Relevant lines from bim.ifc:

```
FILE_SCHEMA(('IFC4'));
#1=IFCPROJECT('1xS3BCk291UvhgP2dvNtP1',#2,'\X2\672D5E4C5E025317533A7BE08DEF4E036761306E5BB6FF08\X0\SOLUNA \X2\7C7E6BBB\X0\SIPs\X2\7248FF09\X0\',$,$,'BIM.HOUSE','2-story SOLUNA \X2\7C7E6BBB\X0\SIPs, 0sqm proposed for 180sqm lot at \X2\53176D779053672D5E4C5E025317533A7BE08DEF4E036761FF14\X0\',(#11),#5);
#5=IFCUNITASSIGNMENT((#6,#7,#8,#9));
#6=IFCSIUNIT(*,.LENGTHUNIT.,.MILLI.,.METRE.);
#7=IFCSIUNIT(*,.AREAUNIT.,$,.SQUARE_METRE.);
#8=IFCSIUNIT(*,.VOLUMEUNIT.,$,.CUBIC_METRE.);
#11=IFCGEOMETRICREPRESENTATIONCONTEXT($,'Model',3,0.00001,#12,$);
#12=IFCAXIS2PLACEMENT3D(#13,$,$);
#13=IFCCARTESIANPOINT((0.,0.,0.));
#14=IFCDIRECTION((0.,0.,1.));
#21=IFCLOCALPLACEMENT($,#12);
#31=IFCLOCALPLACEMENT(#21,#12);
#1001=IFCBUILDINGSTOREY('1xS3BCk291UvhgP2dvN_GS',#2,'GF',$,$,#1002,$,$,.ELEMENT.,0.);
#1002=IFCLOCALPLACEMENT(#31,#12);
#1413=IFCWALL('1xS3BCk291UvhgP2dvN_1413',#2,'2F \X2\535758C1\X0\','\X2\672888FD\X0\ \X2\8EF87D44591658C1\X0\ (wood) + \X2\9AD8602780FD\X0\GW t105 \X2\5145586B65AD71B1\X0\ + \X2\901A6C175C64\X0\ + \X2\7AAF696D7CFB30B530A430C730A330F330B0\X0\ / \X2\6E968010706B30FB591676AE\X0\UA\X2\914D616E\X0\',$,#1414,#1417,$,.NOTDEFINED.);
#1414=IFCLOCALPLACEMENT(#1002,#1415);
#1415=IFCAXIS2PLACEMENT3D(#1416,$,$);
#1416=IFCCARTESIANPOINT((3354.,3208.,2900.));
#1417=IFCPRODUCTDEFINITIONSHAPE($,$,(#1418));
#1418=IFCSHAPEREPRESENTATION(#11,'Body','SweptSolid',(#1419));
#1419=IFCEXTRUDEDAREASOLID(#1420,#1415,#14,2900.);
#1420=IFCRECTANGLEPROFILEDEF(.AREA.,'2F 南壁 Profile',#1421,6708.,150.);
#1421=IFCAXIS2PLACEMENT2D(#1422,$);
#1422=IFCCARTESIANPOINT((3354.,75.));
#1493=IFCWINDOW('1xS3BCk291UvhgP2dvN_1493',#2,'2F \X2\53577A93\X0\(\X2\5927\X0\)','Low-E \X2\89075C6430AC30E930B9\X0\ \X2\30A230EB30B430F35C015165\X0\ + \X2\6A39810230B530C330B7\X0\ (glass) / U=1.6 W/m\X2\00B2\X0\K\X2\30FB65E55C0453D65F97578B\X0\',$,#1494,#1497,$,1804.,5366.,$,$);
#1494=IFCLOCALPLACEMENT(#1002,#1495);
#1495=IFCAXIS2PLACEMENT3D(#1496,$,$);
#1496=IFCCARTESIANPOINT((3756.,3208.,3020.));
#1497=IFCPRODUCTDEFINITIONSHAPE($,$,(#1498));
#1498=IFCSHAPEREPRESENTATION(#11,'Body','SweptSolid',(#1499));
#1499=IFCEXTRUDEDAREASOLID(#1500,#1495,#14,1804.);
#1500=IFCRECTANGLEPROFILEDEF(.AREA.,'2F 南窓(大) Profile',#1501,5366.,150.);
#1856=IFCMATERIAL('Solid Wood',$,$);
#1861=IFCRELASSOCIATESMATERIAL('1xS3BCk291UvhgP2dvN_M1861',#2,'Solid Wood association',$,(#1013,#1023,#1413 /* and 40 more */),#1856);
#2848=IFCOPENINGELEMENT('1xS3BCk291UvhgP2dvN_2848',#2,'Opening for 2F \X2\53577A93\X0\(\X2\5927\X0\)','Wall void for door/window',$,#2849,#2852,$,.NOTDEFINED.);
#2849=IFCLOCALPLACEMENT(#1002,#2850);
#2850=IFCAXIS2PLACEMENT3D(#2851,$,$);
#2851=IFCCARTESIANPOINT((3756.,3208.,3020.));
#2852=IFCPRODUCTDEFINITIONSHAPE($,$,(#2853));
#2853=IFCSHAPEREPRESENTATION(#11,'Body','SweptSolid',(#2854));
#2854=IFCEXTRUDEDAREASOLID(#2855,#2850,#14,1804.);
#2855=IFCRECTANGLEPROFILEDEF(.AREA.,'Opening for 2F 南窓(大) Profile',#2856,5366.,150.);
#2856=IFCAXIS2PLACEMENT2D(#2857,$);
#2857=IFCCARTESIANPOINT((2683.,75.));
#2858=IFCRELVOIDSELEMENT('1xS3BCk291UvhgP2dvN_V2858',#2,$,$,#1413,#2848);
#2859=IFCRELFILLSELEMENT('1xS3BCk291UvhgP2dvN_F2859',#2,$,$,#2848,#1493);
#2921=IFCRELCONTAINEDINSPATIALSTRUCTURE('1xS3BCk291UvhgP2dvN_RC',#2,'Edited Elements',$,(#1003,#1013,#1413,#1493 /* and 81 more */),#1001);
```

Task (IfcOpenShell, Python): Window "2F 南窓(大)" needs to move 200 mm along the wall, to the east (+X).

```python
import ifcopenshell
import ifcopenshell.api.geometry
import ifcopenshell.util.placement

model = ifcopenshell.open("bim.ifc")

window = model.by_guid("1xS3BCk291UvhgP2dvN_1493")
opening = window.FillsVoids[0].RelatingOpeningElement
wall = opening.VoidsElements[0].RelatingBuildingElement

wall_matrix = ifcopenshell.util.placement.get_local_placement(wall.ObjectPlacement)
shift = wall_matrix[:3, 0] * 200.0
before = ifcopenshell.util.placement.get_local_placement(window.ObjectPlacement)[:3, 3].copy()

# The window is not placed relative to its opening, so move both.
for product in (opening, window):
    matrix = ifcopenshell.util.placement.get_local_placement(product.ObjectPlacement)
    matrix[:3, 3] += shift
    ifcopenshell.api.geometry.edit_object_placement(model, product=product, matrix=matrix, is_si=False)

after = ifcopenshell.util.placement.get_local_placement(window.ObjectPlacement)[:3, 3]
print("window moved by", (after - before).round(3) + 0.0)

model.write("bim_v2.ifc")
```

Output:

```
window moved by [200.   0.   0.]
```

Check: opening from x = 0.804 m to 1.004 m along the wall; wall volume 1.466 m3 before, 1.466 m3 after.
